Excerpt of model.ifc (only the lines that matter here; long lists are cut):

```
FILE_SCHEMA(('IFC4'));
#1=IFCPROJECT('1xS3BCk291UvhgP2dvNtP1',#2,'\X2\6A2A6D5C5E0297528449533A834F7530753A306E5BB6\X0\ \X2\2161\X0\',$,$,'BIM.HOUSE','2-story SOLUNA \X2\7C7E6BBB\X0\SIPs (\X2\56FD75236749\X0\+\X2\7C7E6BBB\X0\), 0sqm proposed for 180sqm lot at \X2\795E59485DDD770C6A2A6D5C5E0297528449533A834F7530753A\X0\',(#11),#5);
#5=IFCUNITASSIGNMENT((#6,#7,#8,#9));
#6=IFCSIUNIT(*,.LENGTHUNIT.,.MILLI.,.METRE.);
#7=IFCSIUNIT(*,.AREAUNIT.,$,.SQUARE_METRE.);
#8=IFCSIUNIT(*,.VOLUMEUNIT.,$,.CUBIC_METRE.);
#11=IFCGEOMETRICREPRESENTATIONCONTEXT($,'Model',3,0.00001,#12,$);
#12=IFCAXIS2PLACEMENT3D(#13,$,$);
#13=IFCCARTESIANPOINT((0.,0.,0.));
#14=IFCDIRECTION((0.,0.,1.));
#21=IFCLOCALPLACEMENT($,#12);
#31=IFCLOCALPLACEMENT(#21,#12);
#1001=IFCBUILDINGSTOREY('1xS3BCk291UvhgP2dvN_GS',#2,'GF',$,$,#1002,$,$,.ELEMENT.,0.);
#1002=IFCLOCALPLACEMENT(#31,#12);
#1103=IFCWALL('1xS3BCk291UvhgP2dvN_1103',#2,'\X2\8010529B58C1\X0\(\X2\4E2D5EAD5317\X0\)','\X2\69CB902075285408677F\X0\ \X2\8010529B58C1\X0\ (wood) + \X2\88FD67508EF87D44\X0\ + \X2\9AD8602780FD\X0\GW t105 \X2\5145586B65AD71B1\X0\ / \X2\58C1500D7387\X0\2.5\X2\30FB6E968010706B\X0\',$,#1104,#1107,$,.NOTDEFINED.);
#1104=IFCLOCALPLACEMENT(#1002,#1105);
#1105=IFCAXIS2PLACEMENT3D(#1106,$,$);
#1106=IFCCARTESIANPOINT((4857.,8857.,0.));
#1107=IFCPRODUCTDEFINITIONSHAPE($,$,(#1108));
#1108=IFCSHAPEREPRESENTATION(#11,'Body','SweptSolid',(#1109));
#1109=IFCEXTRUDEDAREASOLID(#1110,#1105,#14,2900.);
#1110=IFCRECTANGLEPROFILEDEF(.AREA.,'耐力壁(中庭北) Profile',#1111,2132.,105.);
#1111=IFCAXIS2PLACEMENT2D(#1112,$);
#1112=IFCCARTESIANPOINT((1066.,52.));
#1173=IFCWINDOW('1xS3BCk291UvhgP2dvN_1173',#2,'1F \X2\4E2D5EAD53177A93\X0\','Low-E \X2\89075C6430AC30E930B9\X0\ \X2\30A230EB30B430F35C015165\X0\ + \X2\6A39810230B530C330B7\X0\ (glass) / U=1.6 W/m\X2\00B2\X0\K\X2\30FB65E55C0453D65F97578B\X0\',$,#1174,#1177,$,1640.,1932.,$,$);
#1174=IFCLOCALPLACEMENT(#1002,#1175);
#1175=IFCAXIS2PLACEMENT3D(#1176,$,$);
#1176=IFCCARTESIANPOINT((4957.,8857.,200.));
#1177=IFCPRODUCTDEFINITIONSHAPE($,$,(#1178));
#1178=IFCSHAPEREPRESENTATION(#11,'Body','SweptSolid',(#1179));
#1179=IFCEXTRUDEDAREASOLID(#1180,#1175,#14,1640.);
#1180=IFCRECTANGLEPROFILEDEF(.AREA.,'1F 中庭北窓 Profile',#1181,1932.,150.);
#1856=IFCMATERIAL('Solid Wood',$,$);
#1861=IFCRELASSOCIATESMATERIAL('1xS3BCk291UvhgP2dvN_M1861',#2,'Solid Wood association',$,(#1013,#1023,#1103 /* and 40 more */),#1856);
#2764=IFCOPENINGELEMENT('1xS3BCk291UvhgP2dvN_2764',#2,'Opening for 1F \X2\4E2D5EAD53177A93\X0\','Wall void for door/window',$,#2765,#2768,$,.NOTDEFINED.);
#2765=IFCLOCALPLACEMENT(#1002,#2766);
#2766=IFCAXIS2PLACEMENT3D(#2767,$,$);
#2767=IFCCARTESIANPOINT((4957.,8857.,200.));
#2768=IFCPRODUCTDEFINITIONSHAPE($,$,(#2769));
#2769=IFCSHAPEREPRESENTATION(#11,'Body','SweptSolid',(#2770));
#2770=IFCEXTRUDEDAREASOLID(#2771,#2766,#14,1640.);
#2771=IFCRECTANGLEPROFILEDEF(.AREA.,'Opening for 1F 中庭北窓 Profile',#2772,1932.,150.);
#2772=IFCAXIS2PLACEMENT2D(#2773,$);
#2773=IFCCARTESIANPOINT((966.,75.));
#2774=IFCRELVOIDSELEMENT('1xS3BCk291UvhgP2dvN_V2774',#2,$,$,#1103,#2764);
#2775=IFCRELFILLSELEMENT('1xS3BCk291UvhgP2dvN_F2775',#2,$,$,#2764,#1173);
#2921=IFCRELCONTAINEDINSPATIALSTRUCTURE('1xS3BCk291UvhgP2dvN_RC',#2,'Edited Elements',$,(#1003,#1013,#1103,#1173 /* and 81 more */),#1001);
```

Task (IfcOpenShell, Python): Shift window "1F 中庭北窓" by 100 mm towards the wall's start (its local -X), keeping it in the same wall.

```python
import ifcopenshell
import ifcopenshell.api.geometry
import ifcopenshell.util.placement

model = ifcopenshell.open("model.ifc")

window = model.by_guid("1xS3BCk291UvhgP2dvN_1173")
opening = window.FillsVoids[0].RelatingOpeningElement
wall = opening.VoidsElements[0].RelatingBuildingElement

wall_matrix = ifcopenshell.util.placement.get_local_placement(wall.ObjectPlacement)
shift = wall_matrix[:3, 0] * -100.0
before = ifcopenshell.util.placement.get_local_placement(window.ObjectPlacement)[:3, 3].copy()

# The window is not placed relative to its opening, so move both.
for product in (opening, window):
    matrix = ifcopenshell.util.placement.get_local_placement(product.ObjectPlacement)
    matrix[:3, 3] += shift
    ifcopenshell.api.geometry.edit_object_placement(model, product=product, matrix=matrix, is_si=False)

after = ifcopenshell.util.placement.get_local_placement(window.ObjectPlacement)[:3, 3]
print("window moved by", (after - before).round(3) + 0.0)

model.write("model_rev.ifc")
```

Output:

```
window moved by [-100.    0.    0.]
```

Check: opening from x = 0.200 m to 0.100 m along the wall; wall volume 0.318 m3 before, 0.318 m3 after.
